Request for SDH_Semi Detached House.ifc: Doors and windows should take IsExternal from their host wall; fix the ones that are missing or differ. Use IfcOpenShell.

First a look at what the model holds.

```python
import ifcopenshell
import ifcopenshell.util.element

model = ifcopenshell.open("SDH_Semi Detached House.ifc")
print(model.schema)
seen = {}
for e in model.by_type("IfcDoor") + model.by_type("IfcWindow"):
    if not e.FillsVoids:
        continue
    host = e.FillsVoids[0].RelatingOpeningElement.VoidsElements[0].RelatingBuildingElement
    own = ifcopenshell.util.element.get_pset(e, f"Pset_{e.is_a()[3:].removesuffix('StandardCase')}Common", "IsExternal")
    wall = ifcopenshell.util.element.get_pset(host, "Pset_WallCommon", "IsExternal")
    seen[e.is_a(), own, wall] = seen.get((e.is_a(), own, wall), 0) + 1
for (cls, own, wall), count in sorted(seen.items(), key=str):
    print(count, cls, "IsExternal:", own, "| host wall:", wall)
```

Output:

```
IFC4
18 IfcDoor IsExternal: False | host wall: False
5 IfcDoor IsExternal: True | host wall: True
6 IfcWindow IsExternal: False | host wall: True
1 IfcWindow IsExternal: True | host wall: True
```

```python
import ifcopenshell
import ifcopenshell.api.pset
import ifcopenshell.util.element

model = ifcopenshell.open("SDH_Semi Detached House.ifc")

count = 0
for ifc_class, pset_name in (("IfcDoor", "Pset_DoorCommon"), ("IfcWindow", "Pset_WindowCommon")):
    for e in model.by_type(ifc_class):
        if not e.FillsVoids:
            continue
        host = e.FillsVoids[0].RelatingOpeningElement.VoidsElements[0].RelatingBuildingElement
        external = ifcopenshell.util.element.get_pset(host, "Pset_WallCommon", "IsExternal")
        if external is None or ifcopenshell.util.element.get_pset(e, pset_name, "IsExternal") == external:
            continue
        pset = ifcopenshell.api.pset.add_pset(model, product=e, name=pset_name)
        ifcopenshell.api.pset.edit_pset(model, pset=pset, properties={"IsExternal": external})
        count += 1

print(count, "updated")

model.write("SDH_Semi Detached House_updated.ifc")
```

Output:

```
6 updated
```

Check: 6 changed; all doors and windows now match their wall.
